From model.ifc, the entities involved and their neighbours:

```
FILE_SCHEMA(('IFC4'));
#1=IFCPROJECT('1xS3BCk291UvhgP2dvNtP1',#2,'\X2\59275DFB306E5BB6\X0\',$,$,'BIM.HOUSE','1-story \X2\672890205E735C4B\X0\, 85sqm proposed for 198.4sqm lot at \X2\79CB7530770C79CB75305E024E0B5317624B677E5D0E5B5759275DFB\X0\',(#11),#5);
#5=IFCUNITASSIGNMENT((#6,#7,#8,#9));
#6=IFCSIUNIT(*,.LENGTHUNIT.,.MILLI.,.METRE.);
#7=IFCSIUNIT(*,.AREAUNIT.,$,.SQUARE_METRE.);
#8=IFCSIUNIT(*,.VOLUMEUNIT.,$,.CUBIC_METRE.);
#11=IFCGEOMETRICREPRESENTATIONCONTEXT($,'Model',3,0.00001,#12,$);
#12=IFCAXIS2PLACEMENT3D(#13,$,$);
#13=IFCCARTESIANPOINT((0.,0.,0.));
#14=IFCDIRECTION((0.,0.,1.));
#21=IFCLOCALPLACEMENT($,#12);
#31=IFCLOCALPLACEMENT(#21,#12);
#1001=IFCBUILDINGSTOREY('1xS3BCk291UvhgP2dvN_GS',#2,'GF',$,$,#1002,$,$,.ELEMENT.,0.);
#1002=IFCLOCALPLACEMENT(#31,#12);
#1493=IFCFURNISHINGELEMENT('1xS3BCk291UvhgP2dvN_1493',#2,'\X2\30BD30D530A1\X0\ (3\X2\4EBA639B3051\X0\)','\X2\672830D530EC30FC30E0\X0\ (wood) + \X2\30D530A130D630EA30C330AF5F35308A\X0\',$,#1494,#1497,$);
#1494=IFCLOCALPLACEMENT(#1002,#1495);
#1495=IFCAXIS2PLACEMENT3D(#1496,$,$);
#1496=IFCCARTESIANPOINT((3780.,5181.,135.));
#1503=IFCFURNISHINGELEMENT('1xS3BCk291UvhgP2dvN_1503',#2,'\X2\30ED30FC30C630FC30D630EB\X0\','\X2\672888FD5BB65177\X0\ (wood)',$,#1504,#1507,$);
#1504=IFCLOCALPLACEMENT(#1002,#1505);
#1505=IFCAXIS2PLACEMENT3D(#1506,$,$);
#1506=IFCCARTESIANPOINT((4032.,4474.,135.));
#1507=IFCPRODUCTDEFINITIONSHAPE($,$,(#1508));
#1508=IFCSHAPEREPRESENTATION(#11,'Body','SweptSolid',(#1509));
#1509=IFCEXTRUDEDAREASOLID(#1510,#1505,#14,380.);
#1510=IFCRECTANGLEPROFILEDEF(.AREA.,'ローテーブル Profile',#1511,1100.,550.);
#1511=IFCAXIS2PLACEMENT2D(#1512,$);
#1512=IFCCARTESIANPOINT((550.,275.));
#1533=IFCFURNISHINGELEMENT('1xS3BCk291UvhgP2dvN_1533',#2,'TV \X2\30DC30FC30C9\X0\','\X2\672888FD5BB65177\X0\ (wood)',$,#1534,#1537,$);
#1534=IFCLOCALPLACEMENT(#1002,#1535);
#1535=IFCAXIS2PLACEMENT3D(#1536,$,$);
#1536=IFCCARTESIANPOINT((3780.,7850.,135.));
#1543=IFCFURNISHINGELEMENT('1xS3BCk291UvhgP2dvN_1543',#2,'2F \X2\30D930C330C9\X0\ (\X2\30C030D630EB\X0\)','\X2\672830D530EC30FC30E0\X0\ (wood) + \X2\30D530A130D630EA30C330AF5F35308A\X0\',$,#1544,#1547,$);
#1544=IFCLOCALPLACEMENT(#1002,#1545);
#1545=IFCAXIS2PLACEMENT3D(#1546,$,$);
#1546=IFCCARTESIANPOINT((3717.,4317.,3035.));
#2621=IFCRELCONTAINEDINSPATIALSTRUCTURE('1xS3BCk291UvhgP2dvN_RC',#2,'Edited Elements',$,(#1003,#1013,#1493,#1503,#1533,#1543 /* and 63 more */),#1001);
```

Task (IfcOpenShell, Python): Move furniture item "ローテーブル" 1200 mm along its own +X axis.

```python
import ifcopenshell
import ifcopenshell.api.geometry
import ifcopenshell.util.placement
import ifcopenshell.util.unit

model = ifcopenshell.open("model.ifc")
unit_scale = ifcopenshell.util.unit.calculate_unit_scale(model)

item = model.by_guid("1xS3BCk291UvhgP2dvN_1503")
matrix = ifcopenshell.util.placement.get_local_placement(item.ObjectPlacement)
matrix[:3, 3] += matrix[:3, 0] * 1.2 / unit_scale
ifcopenshell.api.geometry.edit_object_placement(model, product=item, matrix=matrix, is_si=False)

print(ifcopenshell.util.placement.get_local_placement(item.ObjectPlacement).round(3) + 0.0)

model.write("model_rev.ifc")
```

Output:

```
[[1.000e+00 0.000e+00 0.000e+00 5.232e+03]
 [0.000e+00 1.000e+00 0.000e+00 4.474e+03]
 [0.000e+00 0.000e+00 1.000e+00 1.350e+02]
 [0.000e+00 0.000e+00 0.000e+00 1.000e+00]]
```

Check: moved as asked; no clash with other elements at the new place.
